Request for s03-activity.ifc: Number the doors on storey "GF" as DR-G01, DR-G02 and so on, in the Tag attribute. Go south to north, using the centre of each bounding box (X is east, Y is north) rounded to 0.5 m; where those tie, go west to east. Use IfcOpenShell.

First a look at what the model holds.

```python
import ifcopenshell
import ifcopenshell.util.element
import ifcopenshell.util.placement

model = ifcopenshell.open("s03-activity.ifc")
print(model.schema)
storey = next(s for s in model.by_type("IfcBuildingStorey") if s.Name == "GF")
doors = [e for e in ifcopenshell.util.element.get_decomposition(storey) if e.is_a("IfcDoor")]
for e in sorted(doors, key=lambda e: e.id()):
    origin = ifcopenshell.util.placement.get_local_placement(e.ObjectPlacement)[:3, 3]
    print(e.id(), e.Tag, e.Name, origin.round(2) + 0.0, sep=" | ")
```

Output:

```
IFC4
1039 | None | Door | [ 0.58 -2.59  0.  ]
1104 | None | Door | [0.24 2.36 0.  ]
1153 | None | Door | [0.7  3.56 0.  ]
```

```python
import ifcopenshell
import ifcopenshell.geom
import ifcopenshell.util.element
import ifcopenshell.util.shape

model = ifcopenshell.open("s03-activity.ifc")
settings = ifcopenshell.geom.settings()
settings.set("use-world-coords", True)


def centre(element):
    shape = ifcopenshell.geom.create_shape(settings, element)
    return ifcopenshell.util.shape.get_bbox_centroid(shape.geometry)


storey = next(s for s in model.by_type("IfcBuildingStorey") if s.Name == "GF")
doors = [e for e in ifcopenshell.util.element.get_decomposition(storey) if e.is_a("IfcDoor")]

# Insertion points can sit at a corner or the storey origin, so sort by the geometry (in metres).
centres = {e: centre(e) for e in doors}
doors.sort(key=lambda e: (round(centres[e][1] / 0.5), centres[e][0]))

for i, e in enumerate(doors, start=1):
    number = f"DR-G{i:02d}"
    e.Tag = number
    print(e.id(), number)

model.write("s03-activity-out.ifc")
```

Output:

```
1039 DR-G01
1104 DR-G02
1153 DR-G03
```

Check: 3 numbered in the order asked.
